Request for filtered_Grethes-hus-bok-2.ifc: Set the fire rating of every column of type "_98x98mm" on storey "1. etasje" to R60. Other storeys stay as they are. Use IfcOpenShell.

First a look at what the model holds.

```python
import ifcopenshell
import ifcopenshell.util.element

model = ifcopenshell.open("filtered_Grethes-hus-bok-2.ifc")
print(model.schema)
storey = next(s for s in model.by_type("IfcBuildingStorey") if s.Name == "1. etasje")
columns = [e for e in ifcopenshell.util.element.get_decomposition(storey) if e.is_a("IfcColumn")]
seen = {}
for e in columns:
    element_type = ifcopenshell.util.element.get_type(e)
    key = (element_type.Name if element_type != e and element_type else None, ifcopenshell.util.element.get_pset(e, "Pset_ColumnCommon", "FireRating"))
    seen[key] = seen.get(key, 0) + 1
for (name, value), count in sorted(seen.items(), key=str):
    print(count, "x", name, "|", value)
```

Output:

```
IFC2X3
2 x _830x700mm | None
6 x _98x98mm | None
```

```python
import ifcopenshell
import ifcopenshell.api.pset
import ifcopenshell.util.element

model = ifcopenshell.open("filtered_Grethes-hus-bok-2.ifc")

storey = next(s for s in model.by_type("IfcBuildingStorey") if s.Name == "1. etasje")
columns = [e for e in ifcopenshell.util.element.get_decomposition(storey) if e.is_a("IfcColumn")]

count = 0
for e in columns:
    element_type = ifcopenshell.util.element.get_type(e)
    if element_type in (None, e) or element_type.Name != "_98x98mm":
        continue
    # add_pset returns the element's existing set when there is one.
    pset = ifcopenshell.api.pset.add_pset(model, product=e, name="Pset_ColumnCommon")
    ifcopenshell.api.pset.edit_pset(model, pset=pset, properties={"FireRating": "R60"})
    count += 1

print(count, "columns updated")

model.write("filtered_Grethes-hus-bok-2_edited.ifc")
```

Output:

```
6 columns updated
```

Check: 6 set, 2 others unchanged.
